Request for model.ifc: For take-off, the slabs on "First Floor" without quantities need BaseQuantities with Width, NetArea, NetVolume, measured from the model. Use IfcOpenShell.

First a look at what the model holds.

```python
import ifcopenshell
import ifcopenshell.util.element
import ifcopenshell.util.unit

model = ifcopenshell.open("model.ifc")
print(model.schema)
for unit_type in ("LENGTHUNIT", "AREAUNIT", "VOLUMEUNIT"):
    print(unit_type, ifcopenshell.util.unit.calculate_unit_scale(model, unit_type))
storey = next(s for s in model.by_type("IfcBuildingStorey") if s.Name == "First Floor")
slabs = [e for e in ifcopenshell.util.element.get_decomposition(storey) if e.is_a("IfcSlab")]
for e in sorted(slabs, key=lambda e: e.id()):
    print(e.id(), e.is_a(), e.Name, list(ifcopenshell.util.element.get_psets(e, qtos_only=True)), sep=" | ")
```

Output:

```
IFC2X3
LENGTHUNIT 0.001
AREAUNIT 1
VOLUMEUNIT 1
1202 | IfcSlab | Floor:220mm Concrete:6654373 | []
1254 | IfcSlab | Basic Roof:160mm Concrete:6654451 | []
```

```python
import ifcopenshell
import ifcopenshell.api.pset
import ifcopenshell.geom
import ifcopenshell.util.element
import ifcopenshell.util.shape
import ifcopenshell.util.unit

model = ifcopenshell.open("model.ifc")
unit_scale = ifcopenshell.util.unit.calculate_unit_scale(model)
area_scale = ifcopenshell.util.unit.calculate_unit_scale(model, "AREAUNIT")
volume_scale = ifcopenshell.util.unit.calculate_unit_scale(model, "VOLUMEUNIT")
settings = ifcopenshell.geom.settings()

storey = next(s for s in model.by_type("IfcBuildingStorey") if s.Name == "First Floor")
slabs = [e for e in ifcopenshell.util.element.get_decomposition(storey) if e.is_a("IfcSlab")]

for e in sorted(slabs, key=lambda e: e.id()):
    if ifcopenshell.util.element.get_psets(e, qtos_only=True, should_inherit=False):
        continue
    # Geometry comes back in metres, in the element's own axes.
    shape = ifcopenshell.geom.create_shape(settings, e)
    values = {
        "Width": ifcopenshell.util.shape.get_z(shape.geometry) / unit_scale,
        "NetArea": ifcopenshell.util.shape.get_footprint_area(shape.geometry) / area_scale,
        "NetVolume": ifcopenshell.util.shape.get_volume(shape.geometry) / volume_scale,
    }
    qto = ifcopenshell.api.pset.add_qto(model, product=e, name="BaseQuantities")
    ifcopenshell.api.pset.edit_qto(model, qto=qto, properties=values)
    print(e.id(), {k: round(v, 3) for k, v in values.items()})

model.write("model-out.ifc")
```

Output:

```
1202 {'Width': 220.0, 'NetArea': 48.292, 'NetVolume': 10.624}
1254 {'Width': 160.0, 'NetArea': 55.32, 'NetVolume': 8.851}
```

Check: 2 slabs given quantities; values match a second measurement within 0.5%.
